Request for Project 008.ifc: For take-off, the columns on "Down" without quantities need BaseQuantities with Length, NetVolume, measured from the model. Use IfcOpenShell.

First a look at what the model holds.

```python
import ifcopenshell
import ifcopenshell.util.element
import ifcopenshell.util.unit

model = ifcopenshell.open("Project 008.ifc")
print(model.schema)
for unit_type in ("LENGTHUNIT", "AREAUNIT", "VOLUMEUNIT"):
    print(unit_type, ifcopenshell.util.unit.calculate_unit_scale(model, unit_type))
storey = next(s for s in model.by_type("IfcBuildingStorey") if s.Name == "Down")
columns = [e for e in ifcopenshell.util.element.get_decomposition(storey) if e.is_a("IfcColumn")]
for e in sorted(columns, key=lambda e: e.id()):
    print(e.id(), e.is_a(), e.Name, list(ifcopenshell.util.element.get_psets(e, qtos_only=True)), sep=" | ")
```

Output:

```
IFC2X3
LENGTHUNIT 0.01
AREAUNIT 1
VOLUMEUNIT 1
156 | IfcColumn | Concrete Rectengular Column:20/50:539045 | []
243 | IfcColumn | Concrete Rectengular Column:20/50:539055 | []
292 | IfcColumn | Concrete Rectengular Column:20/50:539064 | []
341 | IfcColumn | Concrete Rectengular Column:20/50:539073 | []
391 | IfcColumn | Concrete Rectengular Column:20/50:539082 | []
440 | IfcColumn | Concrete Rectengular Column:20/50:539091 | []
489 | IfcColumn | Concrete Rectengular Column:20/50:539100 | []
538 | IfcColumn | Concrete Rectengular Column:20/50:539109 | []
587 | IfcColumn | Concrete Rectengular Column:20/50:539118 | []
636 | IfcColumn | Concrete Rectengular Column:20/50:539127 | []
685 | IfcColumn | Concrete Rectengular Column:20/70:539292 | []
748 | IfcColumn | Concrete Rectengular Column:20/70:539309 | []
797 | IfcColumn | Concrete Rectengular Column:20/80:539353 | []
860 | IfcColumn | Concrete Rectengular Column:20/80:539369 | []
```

```python
import ifcopenshell
import ifcopenshell.api.pset
import ifcopenshell.geom
import ifcopenshell.util.element
import ifcopenshell.util.shape
import ifcopenshell.util.unit

model = ifcopenshell.open("Project 008.ifc")
unit_scale = ifcopenshell.util.unit.calculate_unit_scale(model)
volume_scale = ifcopenshell.util.unit.calculate_unit_scale(model, "VOLUMEUNIT")
settings = ifcopenshell.geom.settings()

storey = next(s for s in model.by_type("IfcBuildingStorey") if s.Name == "Down")
columns = [e for e in ifcopenshell.util.element.get_decomposition(storey) if e.is_a("IfcColumn")]

for e in sorted(columns, key=lambda e: e.id()):
    if ifcopenshell.util.element.get_psets(e, qtos_only=True, should_inherit=False):
        continue
    # Geometry comes back in metres, in the element's own axes.
    shape = ifcopenshell.geom.create_shape(settings, e)
    values = {
        "Length": ifcopenshell.util.shape.get_z(shape.geometry) / unit_scale,
        "NetVolume": ifcopenshell.util.shape.get_volume(shape.geometry) / volume_scale,
    }
    qto = ifcopenshell.api.pset.add_qto(model, product=e, name="BaseQuantities")
    ifcopenshell.api.pset.edit_qto(model, qto=qto, properties=values)
    print(e.id(), {k: round(v, 3) for k, v in values.items()})

model.write("Project 008-out.ifc")
```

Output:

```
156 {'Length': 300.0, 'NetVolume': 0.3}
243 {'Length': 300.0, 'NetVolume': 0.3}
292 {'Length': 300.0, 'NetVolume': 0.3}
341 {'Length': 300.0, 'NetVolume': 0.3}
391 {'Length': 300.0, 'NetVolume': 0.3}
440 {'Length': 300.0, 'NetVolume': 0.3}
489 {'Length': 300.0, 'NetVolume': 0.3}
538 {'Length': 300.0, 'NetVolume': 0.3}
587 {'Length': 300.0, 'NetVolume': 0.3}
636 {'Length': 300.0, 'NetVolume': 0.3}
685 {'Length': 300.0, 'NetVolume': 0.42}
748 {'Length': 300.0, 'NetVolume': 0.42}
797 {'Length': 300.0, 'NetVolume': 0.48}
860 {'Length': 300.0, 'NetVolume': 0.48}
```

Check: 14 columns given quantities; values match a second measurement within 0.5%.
